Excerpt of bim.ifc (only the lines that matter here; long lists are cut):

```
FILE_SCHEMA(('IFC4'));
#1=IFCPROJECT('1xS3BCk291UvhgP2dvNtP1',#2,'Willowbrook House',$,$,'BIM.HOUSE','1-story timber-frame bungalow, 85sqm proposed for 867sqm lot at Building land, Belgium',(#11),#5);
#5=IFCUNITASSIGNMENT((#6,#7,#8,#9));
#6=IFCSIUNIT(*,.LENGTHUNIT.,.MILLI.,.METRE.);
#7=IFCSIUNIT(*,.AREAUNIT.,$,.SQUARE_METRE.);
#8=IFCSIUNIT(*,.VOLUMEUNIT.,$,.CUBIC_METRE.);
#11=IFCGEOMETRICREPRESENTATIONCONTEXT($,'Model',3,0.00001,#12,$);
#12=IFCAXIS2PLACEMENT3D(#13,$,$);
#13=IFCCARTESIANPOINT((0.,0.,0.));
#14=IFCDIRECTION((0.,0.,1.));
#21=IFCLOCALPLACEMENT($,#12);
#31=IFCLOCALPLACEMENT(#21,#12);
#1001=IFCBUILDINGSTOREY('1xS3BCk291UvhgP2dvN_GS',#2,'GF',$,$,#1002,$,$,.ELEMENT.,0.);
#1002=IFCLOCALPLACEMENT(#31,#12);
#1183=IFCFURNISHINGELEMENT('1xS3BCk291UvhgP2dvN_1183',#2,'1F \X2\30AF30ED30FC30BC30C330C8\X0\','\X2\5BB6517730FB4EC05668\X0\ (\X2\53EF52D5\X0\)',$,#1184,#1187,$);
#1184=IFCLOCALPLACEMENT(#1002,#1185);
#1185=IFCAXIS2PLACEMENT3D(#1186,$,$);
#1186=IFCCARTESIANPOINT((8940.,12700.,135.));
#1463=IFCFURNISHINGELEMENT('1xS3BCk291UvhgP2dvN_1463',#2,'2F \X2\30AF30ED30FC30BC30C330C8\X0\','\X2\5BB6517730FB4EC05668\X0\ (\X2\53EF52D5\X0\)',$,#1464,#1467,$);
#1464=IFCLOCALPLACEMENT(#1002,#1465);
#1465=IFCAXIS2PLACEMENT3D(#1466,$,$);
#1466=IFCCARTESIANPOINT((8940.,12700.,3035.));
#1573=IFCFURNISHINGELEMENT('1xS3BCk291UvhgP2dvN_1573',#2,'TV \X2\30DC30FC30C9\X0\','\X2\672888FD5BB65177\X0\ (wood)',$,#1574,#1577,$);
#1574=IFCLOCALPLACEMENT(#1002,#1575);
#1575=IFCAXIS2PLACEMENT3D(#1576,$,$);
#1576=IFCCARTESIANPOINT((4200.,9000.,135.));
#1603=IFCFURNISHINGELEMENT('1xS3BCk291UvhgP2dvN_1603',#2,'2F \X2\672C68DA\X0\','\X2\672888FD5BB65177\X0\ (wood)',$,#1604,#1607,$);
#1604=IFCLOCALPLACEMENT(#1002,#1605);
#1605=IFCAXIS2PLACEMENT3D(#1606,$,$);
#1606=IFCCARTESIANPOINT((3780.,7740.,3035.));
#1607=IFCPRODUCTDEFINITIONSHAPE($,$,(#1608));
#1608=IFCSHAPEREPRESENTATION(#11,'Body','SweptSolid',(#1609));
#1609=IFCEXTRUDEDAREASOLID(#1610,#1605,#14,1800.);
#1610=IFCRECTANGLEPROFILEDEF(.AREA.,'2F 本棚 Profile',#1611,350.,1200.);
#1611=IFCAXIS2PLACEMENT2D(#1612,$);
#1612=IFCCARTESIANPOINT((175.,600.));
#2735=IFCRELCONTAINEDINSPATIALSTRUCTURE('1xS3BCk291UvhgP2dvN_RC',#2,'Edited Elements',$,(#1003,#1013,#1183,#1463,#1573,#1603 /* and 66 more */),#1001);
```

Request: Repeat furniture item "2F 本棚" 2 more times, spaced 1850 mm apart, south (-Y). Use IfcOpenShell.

```python
import numpy as np
import ifcopenshell
import ifcopenshell.api.geometry
import ifcopenshell.api.root
import ifcopenshell.util.element
import ifcopenshell.util.placement

model = ifcopenshell.open("bim.ifc")


def reuse_history(source, copy):
    """copy_class also copies each property set's owner history, people and application; keep the originals."""
    for rel in copy.IsDefinedBy:
        if rel.is_a("IfcRelDefinesByProperties") and (history := rel.RelatingPropertyDefinition.OwnerHistory):
            rel.RelatingPropertyDefinition.OwnerHistory = source.OwnerHistory
            ifcopenshell.util.element.remove_deep2(model, history)


source = model.by_guid("1xS3BCk291UvhgP2dvN_1603")
base = ifcopenshell.util.placement.get_local_placement(source.ObjectPlacement)
step = np.array([0.0, -1.0, 0.0]) * 1850.0

for i in range(1, 3):
    copy = ifcopenshell.api.root.copy_class(model, product=source)
    copy.Representation = ifcopenshell.util.element.copy_deep(
        model, source.Representation, exclude=["IfcGeometricRepresentationContext", "IfcRepresentationMap"]
    )
    reuse_history(source, copy)
    matrix = base.copy()
    matrix[:3, 3] += i * step
    print("added at", matrix[:3, 3].round(3) + 0.0)
    ifcopenshell.api.geometry.edit_object_placement(model, product=copy, matrix=matrix, is_si=False)

model.write("bim_v2.ifc")
```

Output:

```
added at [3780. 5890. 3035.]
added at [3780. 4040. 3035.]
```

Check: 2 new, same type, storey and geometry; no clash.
